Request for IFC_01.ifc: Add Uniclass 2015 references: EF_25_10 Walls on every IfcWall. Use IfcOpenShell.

First a look at what the model holds.

```python
import ifcopenshell

model = ifcopenshell.open("IFC_01.ifc")
print(model.schema)
print("classifications:", [c.Name for c in model.by_type("IfcClassification")])
for ifc_class in ("IfcDoor", "IfcRoof", "IfcStair", "IfcWall", "IfcWindow"):
    print(ifc_class, len(model.by_type(ifc_class)))
```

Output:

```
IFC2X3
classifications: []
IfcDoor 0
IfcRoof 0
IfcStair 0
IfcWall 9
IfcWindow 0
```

```python
import ifcopenshell
import ifcopenshell.api.classification

model = ifcopenshell.open("IFC_01.ifc")

# IFC2X3 requires Source and Edition and has no link from the project to the system.
system = model.create_entity("IfcClassification", Source="NBS", Edition="2015", Name="Uniclass 2015")

codes = {
    "IfcWall": ("EF_25_10", "Walls"),
}
for ifc_class, (code, name) in codes.items():
    products = model.by_type(ifc_class)
    ifcopenshell.api.classification.add_reference(
        model, products=products, classification=system, identification=code, name=name
    )
    print(code, len(products))

model.write("IFC_01_rev.ifc")
```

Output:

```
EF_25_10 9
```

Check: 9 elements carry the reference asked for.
